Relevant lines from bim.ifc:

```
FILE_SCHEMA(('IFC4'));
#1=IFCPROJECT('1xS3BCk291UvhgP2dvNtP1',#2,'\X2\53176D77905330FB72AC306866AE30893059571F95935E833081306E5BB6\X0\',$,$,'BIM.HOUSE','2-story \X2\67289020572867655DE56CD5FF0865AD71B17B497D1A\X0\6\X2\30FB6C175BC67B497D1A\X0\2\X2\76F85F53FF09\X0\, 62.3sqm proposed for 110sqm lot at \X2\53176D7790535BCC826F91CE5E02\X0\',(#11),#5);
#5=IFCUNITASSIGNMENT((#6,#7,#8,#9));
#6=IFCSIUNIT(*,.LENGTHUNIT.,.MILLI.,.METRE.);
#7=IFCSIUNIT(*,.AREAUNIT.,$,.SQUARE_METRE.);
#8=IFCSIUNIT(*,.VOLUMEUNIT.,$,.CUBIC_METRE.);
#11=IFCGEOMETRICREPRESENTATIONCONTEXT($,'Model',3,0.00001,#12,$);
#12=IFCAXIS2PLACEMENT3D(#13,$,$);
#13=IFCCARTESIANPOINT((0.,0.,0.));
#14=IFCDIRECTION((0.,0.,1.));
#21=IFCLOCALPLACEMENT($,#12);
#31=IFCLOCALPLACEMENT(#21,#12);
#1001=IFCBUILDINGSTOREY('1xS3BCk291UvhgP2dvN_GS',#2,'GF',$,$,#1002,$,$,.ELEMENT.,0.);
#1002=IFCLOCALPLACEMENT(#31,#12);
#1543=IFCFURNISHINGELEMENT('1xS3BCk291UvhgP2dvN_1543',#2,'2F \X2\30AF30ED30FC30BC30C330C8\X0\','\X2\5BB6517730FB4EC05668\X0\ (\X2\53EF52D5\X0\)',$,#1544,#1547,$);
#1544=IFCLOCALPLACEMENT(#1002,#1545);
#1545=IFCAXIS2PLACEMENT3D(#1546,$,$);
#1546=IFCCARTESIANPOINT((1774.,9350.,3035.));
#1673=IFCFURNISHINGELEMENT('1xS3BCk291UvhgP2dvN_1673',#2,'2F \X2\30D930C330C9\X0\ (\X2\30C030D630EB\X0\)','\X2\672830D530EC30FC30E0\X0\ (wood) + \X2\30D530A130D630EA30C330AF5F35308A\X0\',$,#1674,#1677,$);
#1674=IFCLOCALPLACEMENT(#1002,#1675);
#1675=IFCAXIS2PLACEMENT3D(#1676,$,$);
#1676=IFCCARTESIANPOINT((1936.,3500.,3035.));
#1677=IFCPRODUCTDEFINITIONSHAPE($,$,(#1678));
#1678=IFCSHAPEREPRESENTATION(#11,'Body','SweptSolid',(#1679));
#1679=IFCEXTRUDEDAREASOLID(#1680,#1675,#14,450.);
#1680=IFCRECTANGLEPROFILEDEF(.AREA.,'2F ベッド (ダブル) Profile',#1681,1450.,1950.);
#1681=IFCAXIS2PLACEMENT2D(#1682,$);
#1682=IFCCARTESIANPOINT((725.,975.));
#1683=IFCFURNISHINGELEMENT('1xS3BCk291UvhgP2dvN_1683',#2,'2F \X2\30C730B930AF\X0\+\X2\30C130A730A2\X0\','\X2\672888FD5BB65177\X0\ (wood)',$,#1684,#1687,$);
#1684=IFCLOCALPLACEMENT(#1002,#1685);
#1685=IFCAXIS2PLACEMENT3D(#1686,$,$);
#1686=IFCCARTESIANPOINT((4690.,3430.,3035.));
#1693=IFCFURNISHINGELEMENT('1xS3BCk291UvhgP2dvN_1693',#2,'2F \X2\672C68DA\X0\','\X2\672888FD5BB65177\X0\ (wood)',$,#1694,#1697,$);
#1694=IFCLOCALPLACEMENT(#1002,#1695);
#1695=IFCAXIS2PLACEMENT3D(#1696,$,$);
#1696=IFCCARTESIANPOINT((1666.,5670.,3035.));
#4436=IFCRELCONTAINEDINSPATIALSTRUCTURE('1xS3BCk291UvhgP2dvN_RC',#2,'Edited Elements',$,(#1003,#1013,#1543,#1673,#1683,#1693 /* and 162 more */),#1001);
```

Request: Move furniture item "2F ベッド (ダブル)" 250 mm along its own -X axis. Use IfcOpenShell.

```python
import ifcopenshell
import ifcopenshell.api.geometry
import ifcopenshell.util.placement
import ifcopenshell.util.unit

model = ifcopenshell.open("bim.ifc")
unit_scale = ifcopenshell.util.unit.calculate_unit_scale(model)

item = model.by_id(1673)
matrix = ifcopenshell.util.placement.get_local_placement(item.ObjectPlacement)
matrix[:3, 3] -= matrix[:3, 0] * 0.25 / unit_scale
ifcopenshell.api.geometry.edit_object_placement(model, product=item, matrix=matrix, is_si=False)

print(ifcopenshell.util.placement.get_local_placement(item.ObjectPlacement).round(3) + 0.0)

model.write("bim_updated.ifc")
```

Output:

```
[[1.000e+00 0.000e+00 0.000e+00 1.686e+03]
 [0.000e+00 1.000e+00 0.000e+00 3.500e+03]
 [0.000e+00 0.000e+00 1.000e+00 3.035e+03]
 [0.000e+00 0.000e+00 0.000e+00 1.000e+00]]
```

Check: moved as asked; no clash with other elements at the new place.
